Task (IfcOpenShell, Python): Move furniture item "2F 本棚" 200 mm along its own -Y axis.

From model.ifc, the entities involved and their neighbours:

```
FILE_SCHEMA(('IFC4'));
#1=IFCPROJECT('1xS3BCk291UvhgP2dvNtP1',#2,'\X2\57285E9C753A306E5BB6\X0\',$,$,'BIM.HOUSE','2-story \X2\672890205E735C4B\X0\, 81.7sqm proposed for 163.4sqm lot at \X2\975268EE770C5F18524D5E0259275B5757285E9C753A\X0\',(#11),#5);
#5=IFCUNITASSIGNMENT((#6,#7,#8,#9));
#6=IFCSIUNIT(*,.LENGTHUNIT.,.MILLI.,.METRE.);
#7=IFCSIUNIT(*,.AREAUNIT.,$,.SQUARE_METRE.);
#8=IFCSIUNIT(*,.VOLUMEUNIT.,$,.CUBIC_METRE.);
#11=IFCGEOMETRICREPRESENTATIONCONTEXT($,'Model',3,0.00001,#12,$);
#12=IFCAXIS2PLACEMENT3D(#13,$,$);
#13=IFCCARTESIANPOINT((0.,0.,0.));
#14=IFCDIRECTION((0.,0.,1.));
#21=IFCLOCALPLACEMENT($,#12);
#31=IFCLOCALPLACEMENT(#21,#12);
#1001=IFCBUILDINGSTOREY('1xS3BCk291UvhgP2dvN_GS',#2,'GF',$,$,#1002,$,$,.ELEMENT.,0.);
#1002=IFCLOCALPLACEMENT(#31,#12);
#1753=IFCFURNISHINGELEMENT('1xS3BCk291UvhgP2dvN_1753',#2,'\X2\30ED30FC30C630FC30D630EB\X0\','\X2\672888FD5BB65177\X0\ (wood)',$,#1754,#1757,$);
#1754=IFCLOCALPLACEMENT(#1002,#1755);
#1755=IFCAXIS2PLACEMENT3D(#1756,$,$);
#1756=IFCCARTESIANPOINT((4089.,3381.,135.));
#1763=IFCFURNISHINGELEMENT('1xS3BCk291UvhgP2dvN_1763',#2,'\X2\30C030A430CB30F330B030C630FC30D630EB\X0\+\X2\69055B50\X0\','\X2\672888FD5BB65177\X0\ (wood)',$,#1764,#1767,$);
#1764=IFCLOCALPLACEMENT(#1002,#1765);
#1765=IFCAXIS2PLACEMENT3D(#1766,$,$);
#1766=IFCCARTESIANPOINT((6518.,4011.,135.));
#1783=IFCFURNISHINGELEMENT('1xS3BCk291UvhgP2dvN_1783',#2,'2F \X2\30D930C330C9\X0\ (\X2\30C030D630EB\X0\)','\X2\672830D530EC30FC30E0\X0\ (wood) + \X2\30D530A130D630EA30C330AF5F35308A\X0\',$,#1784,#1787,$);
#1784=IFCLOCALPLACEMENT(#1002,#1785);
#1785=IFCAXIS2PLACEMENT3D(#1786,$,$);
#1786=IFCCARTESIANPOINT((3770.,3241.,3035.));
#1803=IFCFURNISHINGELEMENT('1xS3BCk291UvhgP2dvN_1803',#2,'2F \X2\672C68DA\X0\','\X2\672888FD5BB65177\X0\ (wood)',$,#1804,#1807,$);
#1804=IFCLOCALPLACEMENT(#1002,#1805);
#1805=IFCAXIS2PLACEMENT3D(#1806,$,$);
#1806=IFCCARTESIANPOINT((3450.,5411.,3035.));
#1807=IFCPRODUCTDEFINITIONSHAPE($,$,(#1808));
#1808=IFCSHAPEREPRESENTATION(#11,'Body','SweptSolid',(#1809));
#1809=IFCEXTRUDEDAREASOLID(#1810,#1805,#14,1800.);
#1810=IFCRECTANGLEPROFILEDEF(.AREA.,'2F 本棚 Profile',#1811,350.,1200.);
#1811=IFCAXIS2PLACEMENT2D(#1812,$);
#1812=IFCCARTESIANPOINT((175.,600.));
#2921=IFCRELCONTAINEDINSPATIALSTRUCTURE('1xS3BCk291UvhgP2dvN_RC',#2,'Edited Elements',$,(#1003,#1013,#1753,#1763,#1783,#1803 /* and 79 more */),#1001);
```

```python
import ifcopenshell
import ifcopenshell.api.geometry
import ifcopenshell.util.placement
import ifcopenshell.util.unit

model = ifcopenshell.open("model.ifc")
unit_scale = ifcopenshell.util.unit.calculate_unit_scale(model)

item = model.by_guid("1xS3BCk291UvhgP2dvN_1803")
matrix = ifcopenshell.util.placement.get_local_placement(item.ObjectPlacement)
matrix[:3, 3] -= matrix[:3, 1] * 0.2 / unit_scale
ifcopenshell.api.geometry.edit_object_placement(model, product=item, matrix=matrix, is_si=False)

print(ifcopenshell.util.placement.get_local_placement(item.ObjectPlacement).round(3) + 0.0)

model.write("model_updated.ifc")
```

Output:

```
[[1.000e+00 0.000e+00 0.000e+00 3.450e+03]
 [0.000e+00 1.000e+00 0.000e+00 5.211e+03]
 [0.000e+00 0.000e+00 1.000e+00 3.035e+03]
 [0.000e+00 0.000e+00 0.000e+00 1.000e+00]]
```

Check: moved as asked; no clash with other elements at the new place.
